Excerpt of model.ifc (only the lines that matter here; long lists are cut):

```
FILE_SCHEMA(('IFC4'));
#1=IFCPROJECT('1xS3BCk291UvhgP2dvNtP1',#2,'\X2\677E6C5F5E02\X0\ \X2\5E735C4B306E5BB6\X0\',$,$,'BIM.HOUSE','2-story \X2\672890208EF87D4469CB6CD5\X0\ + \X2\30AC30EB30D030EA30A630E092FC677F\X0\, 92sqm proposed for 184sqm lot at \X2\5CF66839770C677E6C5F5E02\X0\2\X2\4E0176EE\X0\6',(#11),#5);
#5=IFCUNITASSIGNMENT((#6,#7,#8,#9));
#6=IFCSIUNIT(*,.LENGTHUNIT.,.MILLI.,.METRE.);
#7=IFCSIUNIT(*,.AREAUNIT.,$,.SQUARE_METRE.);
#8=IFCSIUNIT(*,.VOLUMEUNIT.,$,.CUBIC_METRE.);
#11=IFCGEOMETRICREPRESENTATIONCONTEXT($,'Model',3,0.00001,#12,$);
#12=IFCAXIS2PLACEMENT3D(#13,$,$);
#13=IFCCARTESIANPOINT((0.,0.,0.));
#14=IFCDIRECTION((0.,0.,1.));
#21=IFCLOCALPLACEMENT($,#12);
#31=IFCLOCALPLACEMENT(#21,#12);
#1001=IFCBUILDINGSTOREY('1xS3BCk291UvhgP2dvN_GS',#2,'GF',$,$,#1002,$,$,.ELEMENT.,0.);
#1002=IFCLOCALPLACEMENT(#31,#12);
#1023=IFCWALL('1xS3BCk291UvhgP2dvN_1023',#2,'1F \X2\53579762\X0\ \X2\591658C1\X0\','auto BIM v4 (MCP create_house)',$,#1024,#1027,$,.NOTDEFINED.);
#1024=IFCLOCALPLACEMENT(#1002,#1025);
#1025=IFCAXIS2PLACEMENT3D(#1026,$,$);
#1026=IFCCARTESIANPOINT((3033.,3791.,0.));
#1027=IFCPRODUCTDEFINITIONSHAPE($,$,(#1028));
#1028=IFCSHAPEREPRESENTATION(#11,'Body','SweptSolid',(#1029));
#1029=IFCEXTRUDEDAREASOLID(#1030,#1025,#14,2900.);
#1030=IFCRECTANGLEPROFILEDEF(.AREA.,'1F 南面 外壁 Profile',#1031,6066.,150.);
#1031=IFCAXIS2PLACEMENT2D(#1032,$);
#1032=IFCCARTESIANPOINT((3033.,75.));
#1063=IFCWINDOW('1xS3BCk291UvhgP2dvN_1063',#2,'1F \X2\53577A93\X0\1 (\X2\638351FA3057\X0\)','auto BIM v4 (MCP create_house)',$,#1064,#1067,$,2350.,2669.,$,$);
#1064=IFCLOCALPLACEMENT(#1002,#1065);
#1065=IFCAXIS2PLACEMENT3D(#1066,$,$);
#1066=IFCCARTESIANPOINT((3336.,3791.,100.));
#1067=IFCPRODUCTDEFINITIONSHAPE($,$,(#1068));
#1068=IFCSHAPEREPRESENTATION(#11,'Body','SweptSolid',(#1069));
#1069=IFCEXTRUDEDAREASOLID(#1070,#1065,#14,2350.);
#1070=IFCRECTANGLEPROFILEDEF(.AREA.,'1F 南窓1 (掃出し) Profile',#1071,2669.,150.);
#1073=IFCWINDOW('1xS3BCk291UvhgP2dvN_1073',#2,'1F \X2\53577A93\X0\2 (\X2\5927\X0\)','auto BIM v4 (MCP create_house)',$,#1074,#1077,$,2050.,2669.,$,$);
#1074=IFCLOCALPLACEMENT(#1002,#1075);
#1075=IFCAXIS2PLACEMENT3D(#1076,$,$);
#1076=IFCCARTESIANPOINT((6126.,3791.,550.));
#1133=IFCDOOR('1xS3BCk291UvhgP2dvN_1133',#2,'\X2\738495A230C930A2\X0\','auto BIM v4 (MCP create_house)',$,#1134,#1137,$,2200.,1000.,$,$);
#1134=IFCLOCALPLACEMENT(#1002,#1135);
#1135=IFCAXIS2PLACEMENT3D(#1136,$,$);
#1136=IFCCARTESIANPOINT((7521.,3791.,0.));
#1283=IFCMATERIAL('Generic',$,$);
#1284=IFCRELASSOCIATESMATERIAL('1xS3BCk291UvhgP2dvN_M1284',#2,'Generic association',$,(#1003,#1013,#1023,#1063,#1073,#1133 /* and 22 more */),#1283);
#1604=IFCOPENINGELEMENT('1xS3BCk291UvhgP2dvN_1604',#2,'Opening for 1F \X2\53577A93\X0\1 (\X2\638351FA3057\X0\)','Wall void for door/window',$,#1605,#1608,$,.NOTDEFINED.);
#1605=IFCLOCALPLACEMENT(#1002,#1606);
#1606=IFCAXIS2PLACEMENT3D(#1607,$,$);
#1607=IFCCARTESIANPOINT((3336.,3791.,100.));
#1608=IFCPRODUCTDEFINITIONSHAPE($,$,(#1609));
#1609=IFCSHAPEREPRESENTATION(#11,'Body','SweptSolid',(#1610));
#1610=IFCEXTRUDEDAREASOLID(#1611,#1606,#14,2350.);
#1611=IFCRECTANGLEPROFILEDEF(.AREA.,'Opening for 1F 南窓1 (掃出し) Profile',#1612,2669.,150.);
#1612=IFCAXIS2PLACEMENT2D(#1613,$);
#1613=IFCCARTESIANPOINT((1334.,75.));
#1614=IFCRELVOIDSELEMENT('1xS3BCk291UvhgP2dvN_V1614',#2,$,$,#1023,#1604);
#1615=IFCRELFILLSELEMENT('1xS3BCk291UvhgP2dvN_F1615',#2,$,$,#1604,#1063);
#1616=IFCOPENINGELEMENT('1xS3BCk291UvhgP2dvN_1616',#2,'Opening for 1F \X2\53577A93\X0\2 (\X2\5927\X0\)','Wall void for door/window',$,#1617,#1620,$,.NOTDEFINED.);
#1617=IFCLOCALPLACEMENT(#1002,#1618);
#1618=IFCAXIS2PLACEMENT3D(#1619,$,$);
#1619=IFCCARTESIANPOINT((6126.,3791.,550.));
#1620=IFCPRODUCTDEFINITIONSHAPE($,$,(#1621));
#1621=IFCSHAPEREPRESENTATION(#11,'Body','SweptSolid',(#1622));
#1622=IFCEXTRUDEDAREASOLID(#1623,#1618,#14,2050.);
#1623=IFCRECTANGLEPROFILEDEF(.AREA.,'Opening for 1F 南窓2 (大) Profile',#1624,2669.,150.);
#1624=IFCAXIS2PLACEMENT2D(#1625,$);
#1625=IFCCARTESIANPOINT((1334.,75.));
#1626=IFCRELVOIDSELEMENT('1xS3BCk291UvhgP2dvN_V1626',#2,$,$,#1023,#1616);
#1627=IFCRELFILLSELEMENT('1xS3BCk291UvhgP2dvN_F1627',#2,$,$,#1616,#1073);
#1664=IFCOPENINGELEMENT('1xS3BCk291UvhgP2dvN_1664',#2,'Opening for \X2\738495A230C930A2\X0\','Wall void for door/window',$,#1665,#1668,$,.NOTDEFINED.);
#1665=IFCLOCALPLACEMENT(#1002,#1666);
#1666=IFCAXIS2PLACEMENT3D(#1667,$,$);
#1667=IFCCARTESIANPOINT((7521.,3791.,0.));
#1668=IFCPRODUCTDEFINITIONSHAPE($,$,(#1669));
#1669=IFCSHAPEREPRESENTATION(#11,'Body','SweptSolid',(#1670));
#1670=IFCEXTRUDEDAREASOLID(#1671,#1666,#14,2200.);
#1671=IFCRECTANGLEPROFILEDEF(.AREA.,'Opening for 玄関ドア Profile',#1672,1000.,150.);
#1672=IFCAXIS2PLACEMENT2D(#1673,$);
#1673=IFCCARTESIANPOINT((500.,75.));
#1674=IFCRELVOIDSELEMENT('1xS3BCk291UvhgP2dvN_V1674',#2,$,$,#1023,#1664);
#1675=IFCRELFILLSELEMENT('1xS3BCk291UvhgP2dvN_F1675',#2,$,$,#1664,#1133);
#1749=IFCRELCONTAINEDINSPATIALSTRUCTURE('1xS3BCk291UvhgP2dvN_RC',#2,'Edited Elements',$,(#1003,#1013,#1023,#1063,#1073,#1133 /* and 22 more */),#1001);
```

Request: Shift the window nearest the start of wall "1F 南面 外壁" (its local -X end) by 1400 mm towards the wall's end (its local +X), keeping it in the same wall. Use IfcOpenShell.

```python
import ifcopenshell
import ifcopenshell.api.geometry
import ifcopenshell.util.placement
import ifcopenshell.util.unit

model = ifcopenshell.open("model.ifc")
unit_scale = ifcopenshell.util.unit.calculate_unit_scale(model)

window = model.by_guid("1xS3BCk291UvhgP2dvN_1063")
opening = window.FillsVoids[0].RelatingOpeningElement
wall = opening.VoidsElements[0].RelatingBuildingElement

wall_matrix = ifcopenshell.util.placement.get_local_placement(wall.ObjectPlacement)
shift = wall_matrix[:3, 0] * 1.4 / unit_scale
before = ifcopenshell.util.placement.get_local_placement(window.ObjectPlacement)[:3, 3].copy()

# The window is not placed relative to its opening, so move both.
for product in (opening, window):
    matrix = ifcopenshell.util.placement.get_local_placement(product.ObjectPlacement)
    matrix[:3, 3] += shift
    ifcopenshell.api.geometry.edit_object_placement(model, product=product, matrix=matrix, is_si=False)

after = ifcopenshell.util.placement.get_local_placement(window.ObjectPlacement)[:3, 3]
print("window moved by", (after - before).round(3) + 0.0)

model.write("model_rev.ifc")
```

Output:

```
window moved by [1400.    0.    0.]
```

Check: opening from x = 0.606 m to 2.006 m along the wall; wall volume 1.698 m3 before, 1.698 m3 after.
